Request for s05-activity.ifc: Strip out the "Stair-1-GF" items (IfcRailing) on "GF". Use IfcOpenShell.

First a look at what the model holds.

```python
import ifcopenshell
import ifcopenshell.util.element

model = ifcopenshell.open("s05-activity.ifc")
print(model.schema)
storey = next(s for s in model.by_type("IfcBuildingStorey") if s.Name == "GF")
railings = [e for e in ifcopenshell.util.element.get_decomposition(storey) if e.is_a("IfcRailing")]
seen = {}
for e in railings:
    element_type = ifcopenshell.util.element.get_type(e)
    name = element_type.Name if element_type not in (None, e) else None
    seen[name] = seen.get(name, 0) + 1
for name, count in sorted(seen.items(), key=str):
    print(count, "x", name)
```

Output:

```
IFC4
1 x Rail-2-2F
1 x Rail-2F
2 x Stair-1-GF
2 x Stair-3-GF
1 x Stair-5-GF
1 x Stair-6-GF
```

```python
import ifcopenshell
import ifcopenshell.api.root
import ifcopenshell.util.element

model = ifcopenshell.open("s05-activity.ifc")

storey = next(s for s in model.by_type("IfcBuildingStorey") if s.Name == "GF")
railings = [e for e in ifcopenshell.util.element.get_decomposition(storey) if e.is_a("IfcRailing")]
targets = [e for e in railings if (t := ifcopenshell.util.element.get_type(e)) not in (None, e) and t.Name == "Stair-1-GF"]

for e in targets:
    ifcopenshell.api.root.remove_product(model, product=e)
print(len(targets), "removed")

model.write("s05-activity_edited.ifc")
```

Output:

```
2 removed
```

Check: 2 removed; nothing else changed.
